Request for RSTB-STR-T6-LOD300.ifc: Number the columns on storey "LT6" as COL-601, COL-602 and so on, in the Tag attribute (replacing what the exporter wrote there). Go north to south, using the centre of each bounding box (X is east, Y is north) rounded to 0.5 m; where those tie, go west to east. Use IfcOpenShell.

First a look at what the model holds.

```python
import ifcopenshell
import ifcopenshell.util.element
import ifcopenshell.util.placement

model = ifcopenshell.open("RSTB-STR-T6-LOD300.ifc")
print(model.schema)
storey = next(s for s in model.by_type("IfcBuildingStorey") if s.Name == "LT6")
columns = [e for e in ifcopenshell.util.element.get_decomposition(storey) if e.is_a("IfcColumn")]
for e in sorted(columns, key=lambda e: e.id()):
    origin = ifcopenshell.util.placement.get_local_placement(e.ObjectPlacement)[:3, 3]
    print(e.id(), e.Tag, e.Name, origin.round(2) + 0.0, sep=" | ")
```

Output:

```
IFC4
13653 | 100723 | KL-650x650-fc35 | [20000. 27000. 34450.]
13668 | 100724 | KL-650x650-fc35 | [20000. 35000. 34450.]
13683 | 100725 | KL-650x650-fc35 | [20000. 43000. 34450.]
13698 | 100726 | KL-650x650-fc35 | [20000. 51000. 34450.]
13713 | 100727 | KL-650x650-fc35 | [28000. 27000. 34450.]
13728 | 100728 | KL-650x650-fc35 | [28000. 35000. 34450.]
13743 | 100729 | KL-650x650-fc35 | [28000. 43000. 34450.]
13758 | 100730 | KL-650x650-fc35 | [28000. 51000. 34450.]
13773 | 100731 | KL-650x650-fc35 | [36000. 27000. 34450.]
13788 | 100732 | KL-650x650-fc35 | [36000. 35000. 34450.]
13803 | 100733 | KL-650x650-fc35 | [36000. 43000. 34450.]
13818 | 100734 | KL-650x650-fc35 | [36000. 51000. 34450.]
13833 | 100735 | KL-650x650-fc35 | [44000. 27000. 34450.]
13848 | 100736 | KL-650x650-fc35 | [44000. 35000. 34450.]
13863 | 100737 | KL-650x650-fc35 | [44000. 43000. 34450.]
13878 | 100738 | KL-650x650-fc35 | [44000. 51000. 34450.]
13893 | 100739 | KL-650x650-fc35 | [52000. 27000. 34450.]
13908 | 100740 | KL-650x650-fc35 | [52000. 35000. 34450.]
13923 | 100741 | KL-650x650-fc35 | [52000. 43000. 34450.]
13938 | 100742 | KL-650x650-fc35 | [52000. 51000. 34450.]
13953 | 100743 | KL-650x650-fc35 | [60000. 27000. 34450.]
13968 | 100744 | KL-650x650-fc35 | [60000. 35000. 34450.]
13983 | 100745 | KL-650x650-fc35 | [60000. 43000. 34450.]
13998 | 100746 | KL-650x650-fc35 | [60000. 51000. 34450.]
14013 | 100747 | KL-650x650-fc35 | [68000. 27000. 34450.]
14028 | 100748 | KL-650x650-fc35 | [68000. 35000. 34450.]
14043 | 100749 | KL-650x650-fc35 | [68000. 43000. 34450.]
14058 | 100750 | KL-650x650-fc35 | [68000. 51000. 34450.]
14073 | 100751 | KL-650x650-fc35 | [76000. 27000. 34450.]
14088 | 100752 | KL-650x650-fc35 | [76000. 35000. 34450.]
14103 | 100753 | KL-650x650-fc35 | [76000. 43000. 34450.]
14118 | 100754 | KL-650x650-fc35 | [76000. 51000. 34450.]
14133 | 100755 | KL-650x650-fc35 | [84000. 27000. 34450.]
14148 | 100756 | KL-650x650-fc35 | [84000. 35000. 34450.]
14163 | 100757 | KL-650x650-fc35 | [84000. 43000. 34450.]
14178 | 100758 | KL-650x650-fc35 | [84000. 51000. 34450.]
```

```python
import ifcopenshell
import ifcopenshell.geom
import ifcopenshell.util.element
import ifcopenshell.util.shape

model = ifcopenshell.open("RSTB-STR-T6-LOD300.ifc")
settings = ifcopenshell.geom.settings()
settings.set("use-world-coords", True)


def centre(element):
    shape = ifcopenshell.geom.create_shape(settings, element)
    return ifcopenshell.util.shape.get_bbox_centroid(shape.geometry)


storey = next(s for s in model.by_type("IfcBuildingStorey") if s.Name == "LT6")
columns = [e for e in ifcopenshell.util.element.get_decomposition(storey) if e.is_a("IfcColumn")]

# Insertion points can sit at a corner or the storey origin, so sort by the geometry (in metres).
centres = {e: centre(e) for e in columns}
columns.sort(key=lambda e: (-round(centres[e][1] / 0.5), centres[e][0]))

for i, e in enumerate(columns, start=1):
    number = f"COL-6{i:02d}"
    e.Tag = number
    print(e.id(), number)

model.write("RSTB-STR-T6-LOD300_rev.ifc")
```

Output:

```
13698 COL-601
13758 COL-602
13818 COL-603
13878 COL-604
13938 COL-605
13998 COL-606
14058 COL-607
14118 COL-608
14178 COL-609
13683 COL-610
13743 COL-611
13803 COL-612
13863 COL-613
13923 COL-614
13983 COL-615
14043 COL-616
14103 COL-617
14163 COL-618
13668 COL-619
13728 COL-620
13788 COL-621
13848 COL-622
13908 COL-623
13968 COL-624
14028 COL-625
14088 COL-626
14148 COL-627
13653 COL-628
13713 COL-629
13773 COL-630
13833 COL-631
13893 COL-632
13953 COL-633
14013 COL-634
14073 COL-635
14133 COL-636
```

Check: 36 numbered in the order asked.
